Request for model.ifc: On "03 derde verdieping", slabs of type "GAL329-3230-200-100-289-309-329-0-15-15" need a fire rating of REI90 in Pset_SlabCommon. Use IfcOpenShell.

First a look at what the model holds.

```python
import ifcopenshell
import ifcopenshell.util.element

model = ifcopenshell.open("model.ifc")
print(model.schema)
storey = next(s for s in model.by_type("IfcBuildingStorey") if s.Name == "03 derde verdieping")
slabs = [e for e in ifcopenshell.util.element.get_decomposition(storey) if e.is_a("IfcSlab")]
seen = {}
for e in slabs:
    element_type = ifcopenshell.util.element.get_type(e)
    key = (element_type.Name if element_type != e and element_type else None, ifcopenshell.util.element.get_pset(e, "Pset_SlabCommon", "FireRating"))
    seen[key] = seen.get(key, 0) + 1
for (name, value), count in sorted(seen.items(), key=str):
    print(count, "x", name, "|", value)
```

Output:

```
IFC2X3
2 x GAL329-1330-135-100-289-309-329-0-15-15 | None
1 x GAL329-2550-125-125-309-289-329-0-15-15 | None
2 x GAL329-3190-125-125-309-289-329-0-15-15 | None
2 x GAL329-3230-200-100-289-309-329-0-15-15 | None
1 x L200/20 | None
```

```python
import ifcopenshell
import ifcopenshell.api.pset
import ifcopenshell.util.element

model = ifcopenshell.open("model.ifc")

storey = next(s for s in model.by_type("IfcBuildingStorey") if s.Name == "03 derde verdieping")
slabs = [e for e in ifcopenshell.util.element.get_decomposition(storey) if e.is_a("IfcSlab")]

count = 0
for e in slabs:
    element_type = ifcopenshell.util.element.get_type(e)
    if element_type in (None, e) or element_type.Name != "GAL329-3230-200-100-289-309-329-0-15-15":
        continue
    found = ifcopenshell.util.element.get_pset(e, "Pset_SlabCommon", should_inherit=False)
    if found:
        pset = model.by_id(found["id"])
        if len(ifcopenshell.util.element.get_elements_by_pset(pset)) > 1:
            pset = ifcopenshell.api.pset.unshare_pset(model, products=[e], pset=pset)[0]
    else:
        pset = ifcopenshell.api.pset.add_pset(model, product=e, name="Pset_SlabCommon")
    ifcopenshell.api.pset.edit_pset(model, pset=pset, properties={"FireRating": "REI90"})
    count += 1

print(count, "slabs updated")

model.write("model_rev.ifc")
```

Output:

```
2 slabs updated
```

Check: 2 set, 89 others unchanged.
